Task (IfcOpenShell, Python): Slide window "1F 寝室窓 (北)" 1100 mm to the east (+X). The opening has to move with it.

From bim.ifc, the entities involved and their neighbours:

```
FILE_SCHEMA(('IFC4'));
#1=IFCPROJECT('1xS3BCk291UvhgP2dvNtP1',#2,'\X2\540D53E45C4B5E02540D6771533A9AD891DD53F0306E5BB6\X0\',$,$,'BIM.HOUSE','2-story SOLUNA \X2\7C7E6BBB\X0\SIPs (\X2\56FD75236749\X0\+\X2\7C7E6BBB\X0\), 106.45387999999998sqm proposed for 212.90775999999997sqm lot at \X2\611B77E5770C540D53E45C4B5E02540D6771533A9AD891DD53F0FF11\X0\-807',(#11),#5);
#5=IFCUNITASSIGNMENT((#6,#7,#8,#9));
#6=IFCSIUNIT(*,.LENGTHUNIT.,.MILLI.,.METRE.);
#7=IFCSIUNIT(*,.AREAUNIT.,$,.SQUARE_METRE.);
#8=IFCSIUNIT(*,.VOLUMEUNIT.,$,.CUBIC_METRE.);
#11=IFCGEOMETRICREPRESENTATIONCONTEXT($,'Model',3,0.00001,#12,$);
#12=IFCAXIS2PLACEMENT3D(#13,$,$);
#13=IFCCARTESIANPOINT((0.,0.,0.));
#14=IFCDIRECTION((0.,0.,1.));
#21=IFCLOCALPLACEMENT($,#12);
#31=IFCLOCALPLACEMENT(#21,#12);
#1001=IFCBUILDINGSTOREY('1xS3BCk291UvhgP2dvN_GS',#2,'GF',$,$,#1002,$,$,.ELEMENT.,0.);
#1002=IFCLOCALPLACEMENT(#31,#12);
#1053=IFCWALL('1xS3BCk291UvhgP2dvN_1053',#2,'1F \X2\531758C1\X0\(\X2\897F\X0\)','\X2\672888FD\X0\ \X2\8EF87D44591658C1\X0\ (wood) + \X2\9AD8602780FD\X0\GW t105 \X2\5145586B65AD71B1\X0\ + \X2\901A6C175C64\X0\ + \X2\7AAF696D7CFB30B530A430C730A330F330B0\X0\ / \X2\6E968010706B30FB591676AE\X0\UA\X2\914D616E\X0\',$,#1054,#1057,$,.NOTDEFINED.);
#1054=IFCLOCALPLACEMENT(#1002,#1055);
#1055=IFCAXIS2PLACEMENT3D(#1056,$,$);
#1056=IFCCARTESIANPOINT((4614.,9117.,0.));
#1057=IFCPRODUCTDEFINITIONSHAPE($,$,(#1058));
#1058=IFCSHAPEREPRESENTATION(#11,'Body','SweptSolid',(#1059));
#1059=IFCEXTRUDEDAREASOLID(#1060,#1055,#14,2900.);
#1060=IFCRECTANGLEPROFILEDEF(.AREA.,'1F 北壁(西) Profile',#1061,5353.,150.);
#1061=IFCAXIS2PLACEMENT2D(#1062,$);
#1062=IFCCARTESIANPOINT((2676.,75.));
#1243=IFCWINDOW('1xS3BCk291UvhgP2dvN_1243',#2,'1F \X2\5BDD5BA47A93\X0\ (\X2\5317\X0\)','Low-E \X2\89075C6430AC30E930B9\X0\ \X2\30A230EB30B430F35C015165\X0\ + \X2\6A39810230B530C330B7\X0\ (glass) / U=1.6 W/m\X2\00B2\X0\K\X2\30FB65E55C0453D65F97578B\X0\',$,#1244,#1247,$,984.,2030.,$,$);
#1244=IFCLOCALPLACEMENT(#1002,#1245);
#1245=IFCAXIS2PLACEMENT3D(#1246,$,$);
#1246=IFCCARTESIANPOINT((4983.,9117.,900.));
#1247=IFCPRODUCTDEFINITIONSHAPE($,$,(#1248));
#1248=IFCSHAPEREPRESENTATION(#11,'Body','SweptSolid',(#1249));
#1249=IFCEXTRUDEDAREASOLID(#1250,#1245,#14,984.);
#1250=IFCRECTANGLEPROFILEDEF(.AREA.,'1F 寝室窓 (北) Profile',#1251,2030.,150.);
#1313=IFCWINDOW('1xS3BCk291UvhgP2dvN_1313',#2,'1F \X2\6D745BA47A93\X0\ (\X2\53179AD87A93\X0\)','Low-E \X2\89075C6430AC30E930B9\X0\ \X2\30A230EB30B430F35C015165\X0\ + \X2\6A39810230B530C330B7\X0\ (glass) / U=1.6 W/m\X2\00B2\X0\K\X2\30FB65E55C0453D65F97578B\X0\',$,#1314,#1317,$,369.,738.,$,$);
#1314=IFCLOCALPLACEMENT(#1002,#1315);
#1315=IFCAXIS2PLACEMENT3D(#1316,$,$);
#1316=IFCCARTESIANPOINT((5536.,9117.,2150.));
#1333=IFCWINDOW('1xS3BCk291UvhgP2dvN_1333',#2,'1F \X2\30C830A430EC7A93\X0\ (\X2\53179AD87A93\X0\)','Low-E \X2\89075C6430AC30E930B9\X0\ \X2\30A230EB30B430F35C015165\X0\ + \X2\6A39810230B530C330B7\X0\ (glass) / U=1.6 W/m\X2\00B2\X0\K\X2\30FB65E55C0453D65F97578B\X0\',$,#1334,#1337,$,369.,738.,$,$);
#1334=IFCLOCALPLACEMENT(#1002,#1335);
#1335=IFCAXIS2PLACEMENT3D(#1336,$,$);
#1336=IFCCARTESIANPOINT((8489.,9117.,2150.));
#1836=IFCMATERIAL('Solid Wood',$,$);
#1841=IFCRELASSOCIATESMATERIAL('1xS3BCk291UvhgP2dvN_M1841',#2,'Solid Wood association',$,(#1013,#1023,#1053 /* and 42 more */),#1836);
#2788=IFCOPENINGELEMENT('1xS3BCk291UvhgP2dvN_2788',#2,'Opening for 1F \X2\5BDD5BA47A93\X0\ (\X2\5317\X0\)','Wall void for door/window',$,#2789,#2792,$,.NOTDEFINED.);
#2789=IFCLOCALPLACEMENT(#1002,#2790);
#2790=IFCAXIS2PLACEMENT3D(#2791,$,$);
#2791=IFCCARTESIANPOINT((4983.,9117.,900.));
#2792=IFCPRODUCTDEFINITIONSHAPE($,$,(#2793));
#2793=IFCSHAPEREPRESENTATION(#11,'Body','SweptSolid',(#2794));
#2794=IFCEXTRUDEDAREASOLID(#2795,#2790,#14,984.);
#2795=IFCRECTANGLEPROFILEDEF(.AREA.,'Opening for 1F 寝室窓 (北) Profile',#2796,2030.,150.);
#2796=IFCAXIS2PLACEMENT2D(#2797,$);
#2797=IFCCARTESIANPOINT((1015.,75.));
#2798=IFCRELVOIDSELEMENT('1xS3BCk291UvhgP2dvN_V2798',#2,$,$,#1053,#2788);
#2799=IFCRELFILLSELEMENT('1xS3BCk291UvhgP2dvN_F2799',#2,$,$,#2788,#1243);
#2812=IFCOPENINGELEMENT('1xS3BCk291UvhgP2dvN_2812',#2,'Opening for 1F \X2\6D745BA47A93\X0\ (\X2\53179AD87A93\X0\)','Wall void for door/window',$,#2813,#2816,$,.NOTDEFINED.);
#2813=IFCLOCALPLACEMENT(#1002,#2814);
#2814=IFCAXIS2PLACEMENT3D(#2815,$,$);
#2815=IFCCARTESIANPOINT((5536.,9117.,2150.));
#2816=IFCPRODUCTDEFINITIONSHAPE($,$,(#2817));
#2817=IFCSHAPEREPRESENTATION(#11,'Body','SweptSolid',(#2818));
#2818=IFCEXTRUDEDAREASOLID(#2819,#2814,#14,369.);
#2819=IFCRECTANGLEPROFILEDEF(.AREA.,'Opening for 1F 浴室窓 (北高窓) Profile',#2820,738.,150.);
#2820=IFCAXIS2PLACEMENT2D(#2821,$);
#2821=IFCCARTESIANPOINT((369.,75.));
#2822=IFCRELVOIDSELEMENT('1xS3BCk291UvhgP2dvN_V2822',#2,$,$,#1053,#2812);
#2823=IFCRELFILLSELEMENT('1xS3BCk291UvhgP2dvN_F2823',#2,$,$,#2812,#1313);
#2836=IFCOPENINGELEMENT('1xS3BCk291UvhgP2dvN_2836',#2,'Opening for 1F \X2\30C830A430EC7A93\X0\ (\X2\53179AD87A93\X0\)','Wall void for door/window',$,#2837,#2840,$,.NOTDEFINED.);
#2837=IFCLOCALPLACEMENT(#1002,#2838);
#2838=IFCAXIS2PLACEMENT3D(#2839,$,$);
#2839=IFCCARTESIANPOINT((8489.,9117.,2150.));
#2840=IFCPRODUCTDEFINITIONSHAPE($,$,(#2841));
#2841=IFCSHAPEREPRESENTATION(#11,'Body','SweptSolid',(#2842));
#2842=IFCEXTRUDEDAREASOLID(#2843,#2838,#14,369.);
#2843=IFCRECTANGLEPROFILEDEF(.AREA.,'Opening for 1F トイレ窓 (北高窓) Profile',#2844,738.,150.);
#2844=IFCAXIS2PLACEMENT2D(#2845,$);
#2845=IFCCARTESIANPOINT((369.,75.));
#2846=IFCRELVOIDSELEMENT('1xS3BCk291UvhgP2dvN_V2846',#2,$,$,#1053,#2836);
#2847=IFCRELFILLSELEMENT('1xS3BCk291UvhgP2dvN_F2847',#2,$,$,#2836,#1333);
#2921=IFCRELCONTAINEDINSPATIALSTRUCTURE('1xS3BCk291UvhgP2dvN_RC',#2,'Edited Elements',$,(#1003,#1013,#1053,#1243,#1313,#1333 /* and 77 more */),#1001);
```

```python
import ifcopenshell
import ifcopenshell.api.geometry
import ifcopenshell.util.placement
import ifcopenshell.util.unit

model = ifcopenshell.open("bim.ifc")
unit_scale = ifcopenshell.util.unit.calculate_unit_scale(model)

window = model.by_guid("1xS3BCk291UvhgP2dvN_1243")
opening = window.FillsVoids[0].RelatingOpeningElement
wall = opening.VoidsElements[0].RelatingBuildingElement

wall_matrix = ifcopenshell.util.placement.get_local_placement(wall.ObjectPlacement)
shift = wall_matrix[:3, 0] * 1.1 / unit_scale
before = ifcopenshell.util.placement.get_local_placement(window.ObjectPlacement)[:3, 3].copy()

# The window is not placed relative to its opening, so move both.
for product in (opening, window):
    matrix = ifcopenshell.util.placement.get_local_placement(product.ObjectPlacement)
    matrix[:3, 3] += shift
    ifcopenshell.api.geometry.edit_object_placement(model, product=product, matrix=matrix, is_si=False)

after = ifcopenshell.util.placement.get_local_placement(window.ObjectPlacement)[:3, 3]
print("window moved by", (after - before).round(3) + 0.0)

model.write("bim_updated.ifc")
```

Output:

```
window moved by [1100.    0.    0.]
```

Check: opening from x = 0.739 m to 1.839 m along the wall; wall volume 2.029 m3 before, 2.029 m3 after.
